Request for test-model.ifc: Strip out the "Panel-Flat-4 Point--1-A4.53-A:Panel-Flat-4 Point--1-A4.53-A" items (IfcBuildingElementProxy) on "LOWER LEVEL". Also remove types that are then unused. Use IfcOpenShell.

First a look at what the model holds.

```python
import ifcopenshell
import ifcopenshell.util.element

model = ifcopenshell.open("test-model.ifc")
print(model.schema)
storey = next(s for s in model.by_type("IfcBuildingStorey") if s.Name == "LOWER LEVEL")
proxies = [e for e in ifcopenshell.util.element.get_decomposition(storey) if e.is_a("IfcBuildingElementProxy")]
seen = {}
for e in proxies:
    element_type = ifcopenshell.util.element.get_type(e)
    name = element_type.Name if element_type not in (None, e) else None
    seen[name] = seen.get(name, 0) + 1
for name, count in sorted(seen.items(), key=str):
    print(count, "x", name)
```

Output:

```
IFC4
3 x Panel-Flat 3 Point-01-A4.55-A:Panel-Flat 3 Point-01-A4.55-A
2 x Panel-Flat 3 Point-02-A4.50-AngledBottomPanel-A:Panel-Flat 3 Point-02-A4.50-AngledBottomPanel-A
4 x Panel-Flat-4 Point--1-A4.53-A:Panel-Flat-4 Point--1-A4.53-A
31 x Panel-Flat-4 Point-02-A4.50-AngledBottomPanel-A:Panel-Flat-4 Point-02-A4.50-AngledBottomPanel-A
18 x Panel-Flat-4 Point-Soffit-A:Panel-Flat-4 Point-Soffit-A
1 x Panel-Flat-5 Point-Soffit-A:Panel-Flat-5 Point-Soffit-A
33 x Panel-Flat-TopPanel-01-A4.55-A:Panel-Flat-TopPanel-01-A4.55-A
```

```python
import ifcopenshell
import ifcopenshell.api.root
import ifcopenshell.util.element

model = ifcopenshell.open("test-model.ifc")

storey = next(s for s in model.by_type("IfcBuildingStorey") if s.Name == "LOWER LEVEL")
proxies = [e for e in ifcopenshell.util.element.get_decomposition(storey) if e.is_a("IfcBuildingElementProxy")]
targets = [e for e in proxies if (t := ifcopenshell.util.element.get_type(e)) not in (None, e) and t.Name == "Panel-Flat-4 Point--1-A4.53-A:Panel-Flat-4 Point--1-A4.53-A"]
types = {ifcopenshell.util.element.get_type(e) for e in targets} - {None, *targets}

for e in targets:
    ifcopenshell.api.root.remove_product(model, product=e)
print(len(targets), "removed")

unused = [t for t in types if not ifcopenshell.util.element.get_types(t)]
for t in unused:
    ifcopenshell.api.root.remove_product(model, product=t)
print(len(unused), "unused types removed")

model.write("test-model_v2.ifc")
```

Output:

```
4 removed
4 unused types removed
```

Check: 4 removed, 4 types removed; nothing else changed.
